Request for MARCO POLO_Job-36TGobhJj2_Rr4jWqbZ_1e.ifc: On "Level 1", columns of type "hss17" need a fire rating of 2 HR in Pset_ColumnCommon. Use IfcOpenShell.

First a look at what the model holds.

```python
import ifcopenshell
import ifcopenshell.util.element

model = ifcopenshell.open("MARCO POLO_Job-36TGobhJj2_Rr4jWqbZ_1e.ifc")
print(model.schema)
storey = next(s for s in model.by_type("IfcBuildingStorey") if s.Name == "Level 1")
columns = [e for e in ifcopenshell.util.element.get_decomposition(storey) if e.is_a("IfcColumn")]
seen = {}
for e in columns:
    element_type = ifcopenshell.util.element.get_type(e)
    key = (element_type.Name if element_type != e and element_type else None, ifcopenshell.util.element.get_pset(e, "Pset_ColumnCommon", "FireRating"))
    seen[key] = seen.get(key, 0) + 1
for (name, value), count in sorted(seen.items(), key=str):
    print(count, "x", name, "|", value)
```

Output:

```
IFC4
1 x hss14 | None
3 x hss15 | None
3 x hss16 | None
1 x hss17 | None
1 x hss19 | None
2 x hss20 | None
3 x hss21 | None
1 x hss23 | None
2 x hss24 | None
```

```python
import ifcopenshell
import ifcopenshell.api.pset
import ifcopenshell.util.element

model = ifcopenshell.open("MARCO POLO_Job-36TGobhJj2_Rr4jWqbZ_1e.ifc")

storey = next(s for s in model.by_type("IfcBuildingStorey") if s.Name == "Level 1")
columns = [e for e in ifcopenshell.util.element.get_decomposition(storey) if e.is_a("IfcColumn")]

count = 0
for e in columns:
    element_type = ifcopenshell.util.element.get_type(e)
    if element_type in (None, e) or element_type.Name != "hss17":
        continue
    # add_pset returns the element's existing set when there is one.
    pset = ifcopenshell.api.pset.add_pset(model, product=e, name="Pset_ColumnCommon")
    ifcopenshell.api.pset.edit_pset(model, pset=pset, properties={"FireRating": "2 HR"})
    count += 1

print(count, "columns updated")

model.write("MARCO POLO_Job-36TGobhJj2_Rr4jWqbZ_1e_updated.ifc")
```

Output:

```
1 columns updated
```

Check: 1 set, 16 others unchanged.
